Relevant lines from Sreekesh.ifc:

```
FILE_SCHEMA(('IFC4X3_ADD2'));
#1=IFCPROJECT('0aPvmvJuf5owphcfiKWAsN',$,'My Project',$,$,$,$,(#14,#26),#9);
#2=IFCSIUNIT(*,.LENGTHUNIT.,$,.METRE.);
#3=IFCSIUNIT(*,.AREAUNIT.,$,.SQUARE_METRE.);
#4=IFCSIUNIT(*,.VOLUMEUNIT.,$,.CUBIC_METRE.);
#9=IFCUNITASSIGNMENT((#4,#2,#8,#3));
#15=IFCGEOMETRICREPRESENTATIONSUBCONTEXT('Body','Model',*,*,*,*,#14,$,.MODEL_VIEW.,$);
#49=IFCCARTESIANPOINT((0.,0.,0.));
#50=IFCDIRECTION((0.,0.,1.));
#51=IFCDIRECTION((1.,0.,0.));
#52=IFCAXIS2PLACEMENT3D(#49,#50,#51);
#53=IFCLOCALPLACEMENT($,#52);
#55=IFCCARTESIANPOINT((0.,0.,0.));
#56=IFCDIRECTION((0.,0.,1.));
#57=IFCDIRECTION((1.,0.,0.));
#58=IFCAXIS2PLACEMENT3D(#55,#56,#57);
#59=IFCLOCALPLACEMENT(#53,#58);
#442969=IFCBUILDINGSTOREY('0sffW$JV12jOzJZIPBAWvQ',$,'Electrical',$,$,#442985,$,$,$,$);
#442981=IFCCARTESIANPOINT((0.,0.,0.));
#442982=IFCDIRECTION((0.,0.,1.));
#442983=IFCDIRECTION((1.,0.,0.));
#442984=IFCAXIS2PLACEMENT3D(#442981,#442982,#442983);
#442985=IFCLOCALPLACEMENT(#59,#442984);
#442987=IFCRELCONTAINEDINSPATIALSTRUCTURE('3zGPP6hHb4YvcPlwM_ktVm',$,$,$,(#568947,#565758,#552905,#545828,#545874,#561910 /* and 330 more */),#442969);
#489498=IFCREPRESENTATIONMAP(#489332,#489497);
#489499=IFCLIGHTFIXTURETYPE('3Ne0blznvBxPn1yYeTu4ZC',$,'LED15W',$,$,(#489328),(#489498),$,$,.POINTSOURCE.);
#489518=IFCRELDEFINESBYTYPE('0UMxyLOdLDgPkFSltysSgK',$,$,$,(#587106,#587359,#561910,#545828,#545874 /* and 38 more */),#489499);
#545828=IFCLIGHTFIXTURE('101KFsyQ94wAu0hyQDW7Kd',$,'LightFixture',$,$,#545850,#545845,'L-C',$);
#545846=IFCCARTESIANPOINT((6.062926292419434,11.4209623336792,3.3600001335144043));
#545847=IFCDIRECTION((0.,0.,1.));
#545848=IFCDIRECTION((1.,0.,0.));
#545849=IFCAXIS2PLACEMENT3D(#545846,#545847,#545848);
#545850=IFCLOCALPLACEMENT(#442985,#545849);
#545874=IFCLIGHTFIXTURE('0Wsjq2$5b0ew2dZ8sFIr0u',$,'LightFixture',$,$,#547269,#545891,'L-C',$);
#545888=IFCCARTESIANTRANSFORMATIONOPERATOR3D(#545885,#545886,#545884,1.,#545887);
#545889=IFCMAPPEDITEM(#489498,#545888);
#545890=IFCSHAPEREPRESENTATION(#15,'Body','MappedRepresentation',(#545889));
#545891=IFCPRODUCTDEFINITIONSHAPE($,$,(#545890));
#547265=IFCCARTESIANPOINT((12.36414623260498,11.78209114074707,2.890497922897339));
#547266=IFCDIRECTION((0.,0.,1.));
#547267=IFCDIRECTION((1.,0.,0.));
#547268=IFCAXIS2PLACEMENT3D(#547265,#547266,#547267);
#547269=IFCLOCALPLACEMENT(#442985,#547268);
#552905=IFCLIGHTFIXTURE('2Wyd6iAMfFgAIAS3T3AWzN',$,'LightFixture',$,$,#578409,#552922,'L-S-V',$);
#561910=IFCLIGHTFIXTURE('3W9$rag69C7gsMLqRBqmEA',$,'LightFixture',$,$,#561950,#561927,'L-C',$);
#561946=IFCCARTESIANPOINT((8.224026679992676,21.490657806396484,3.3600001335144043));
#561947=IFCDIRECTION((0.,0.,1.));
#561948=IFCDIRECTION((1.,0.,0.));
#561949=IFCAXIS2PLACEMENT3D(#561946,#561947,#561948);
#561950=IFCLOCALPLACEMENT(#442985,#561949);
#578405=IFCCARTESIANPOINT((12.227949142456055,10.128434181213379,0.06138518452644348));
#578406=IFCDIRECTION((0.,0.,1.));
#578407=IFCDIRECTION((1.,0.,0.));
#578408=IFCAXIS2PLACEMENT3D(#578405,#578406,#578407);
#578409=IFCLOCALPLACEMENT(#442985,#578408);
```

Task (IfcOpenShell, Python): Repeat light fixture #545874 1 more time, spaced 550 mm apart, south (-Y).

```python
import numpy as np
import ifcopenshell
import ifcopenshell.api.geometry
import ifcopenshell.api.root
import ifcopenshell.util.element
import ifcopenshell.util.placement
import ifcopenshell.util.unit

model = ifcopenshell.open("Sreekesh.ifc")
unit_scale = ifcopenshell.util.unit.calculate_unit_scale(model)

source = model.by_guid("0Wsjq2$5b0ew2dZ8sFIr0u")
base = ifcopenshell.util.placement.get_local_placement(source.ObjectPlacement)
step = np.array([0.0, -1.0, 0.0]) * 0.55 / unit_scale

for i in range(1, 2):
    copy = ifcopenshell.api.root.copy_class(model, product=source)
    copy.Representation = ifcopenshell.util.element.copy_deep(
        model, source.Representation, exclude=["IfcGeometricRepresentationContext", "IfcRepresentationMap"]
    )
    copy.Tag = None
    matrix = base.copy()
    matrix[:3, 3] += i * step
    print("added at", matrix[:3, 3].round(3) + 0.0)
    ifcopenshell.api.geometry.edit_object_placement(model, product=copy, matrix=matrix, is_si=False)

model.write("Sreekesh_updated.ifc")
```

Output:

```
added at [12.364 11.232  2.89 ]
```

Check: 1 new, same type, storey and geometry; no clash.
